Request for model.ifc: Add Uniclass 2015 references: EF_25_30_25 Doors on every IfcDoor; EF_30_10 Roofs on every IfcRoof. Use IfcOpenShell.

First a look at what the model holds.

```python
import ifcopenshell

model = ifcopenshell.open("model.ifc")
print(model.schema)
print("classifications:", [c.Name for c in model.by_type("IfcClassification")])
for ifc_class in ("IfcDoor", "IfcRoof", "IfcStair", "IfcWall", "IfcWindow"):
    print(ifc_class, len(model.by_type(ifc_class)))
```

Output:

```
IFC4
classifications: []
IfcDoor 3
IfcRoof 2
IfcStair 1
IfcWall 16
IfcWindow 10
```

```python
import ifcopenshell
import ifcopenshell.api.classification

model = ifcopenshell.open("model.ifc")

system = ifcopenshell.api.classification.add_classification(model, classification="Uniclass 2015")

codes = {
    "IfcDoor": ("EF_25_30_25", "Doors"),
    "IfcRoof": ("EF_30_10", "Roofs"),
}
for ifc_class, (code, name) in codes.items():
    products = model.by_type(ifc_class)
    ifcopenshell.api.classification.add_reference(
        model, products=products, classification=system, identification=code, name=name
    )
    print(code, len(products))

model.write("model_v2.ifc")
```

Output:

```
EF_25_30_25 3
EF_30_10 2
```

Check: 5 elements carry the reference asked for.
